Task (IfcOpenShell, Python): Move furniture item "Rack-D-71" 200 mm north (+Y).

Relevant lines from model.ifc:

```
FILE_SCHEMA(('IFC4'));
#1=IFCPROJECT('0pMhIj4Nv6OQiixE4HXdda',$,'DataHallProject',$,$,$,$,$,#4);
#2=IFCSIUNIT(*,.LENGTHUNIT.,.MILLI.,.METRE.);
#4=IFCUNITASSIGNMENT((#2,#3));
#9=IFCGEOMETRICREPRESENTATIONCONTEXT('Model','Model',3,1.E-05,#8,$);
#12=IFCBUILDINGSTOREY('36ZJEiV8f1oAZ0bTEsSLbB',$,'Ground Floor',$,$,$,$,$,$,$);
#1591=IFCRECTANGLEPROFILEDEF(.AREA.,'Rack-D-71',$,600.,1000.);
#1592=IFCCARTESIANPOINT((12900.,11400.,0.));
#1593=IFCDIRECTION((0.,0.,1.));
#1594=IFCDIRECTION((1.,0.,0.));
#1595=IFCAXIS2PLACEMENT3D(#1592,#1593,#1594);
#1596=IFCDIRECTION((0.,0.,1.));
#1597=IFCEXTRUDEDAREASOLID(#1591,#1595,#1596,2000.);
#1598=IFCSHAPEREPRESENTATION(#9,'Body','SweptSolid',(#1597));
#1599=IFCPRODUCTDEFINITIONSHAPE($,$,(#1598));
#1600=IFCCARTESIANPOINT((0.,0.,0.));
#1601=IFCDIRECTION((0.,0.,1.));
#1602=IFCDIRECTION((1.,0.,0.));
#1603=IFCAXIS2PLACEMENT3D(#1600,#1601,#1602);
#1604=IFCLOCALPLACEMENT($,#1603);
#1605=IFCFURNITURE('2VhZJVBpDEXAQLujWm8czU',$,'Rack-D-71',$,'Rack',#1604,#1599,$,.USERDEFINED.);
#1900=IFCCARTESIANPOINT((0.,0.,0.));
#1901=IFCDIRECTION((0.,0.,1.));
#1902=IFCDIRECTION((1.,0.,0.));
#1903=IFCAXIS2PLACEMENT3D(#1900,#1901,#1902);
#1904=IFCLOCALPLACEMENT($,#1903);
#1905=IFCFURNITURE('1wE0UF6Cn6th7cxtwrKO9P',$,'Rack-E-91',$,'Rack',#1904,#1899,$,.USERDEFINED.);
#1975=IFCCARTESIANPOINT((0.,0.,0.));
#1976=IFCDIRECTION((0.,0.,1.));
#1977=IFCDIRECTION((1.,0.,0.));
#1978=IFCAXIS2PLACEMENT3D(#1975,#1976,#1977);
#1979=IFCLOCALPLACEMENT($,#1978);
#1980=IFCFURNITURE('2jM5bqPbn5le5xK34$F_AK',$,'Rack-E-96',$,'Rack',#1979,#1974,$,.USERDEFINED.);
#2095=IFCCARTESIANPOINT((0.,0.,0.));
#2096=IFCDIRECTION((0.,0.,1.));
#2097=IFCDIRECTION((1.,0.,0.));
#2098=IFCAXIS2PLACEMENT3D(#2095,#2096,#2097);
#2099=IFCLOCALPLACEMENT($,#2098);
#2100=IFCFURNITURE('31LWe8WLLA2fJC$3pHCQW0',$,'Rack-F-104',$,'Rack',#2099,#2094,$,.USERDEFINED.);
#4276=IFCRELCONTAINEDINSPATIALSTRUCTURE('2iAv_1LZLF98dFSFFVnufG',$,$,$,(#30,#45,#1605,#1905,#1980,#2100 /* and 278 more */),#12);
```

```python
import ifcopenshell
import ifcopenshell.api.geometry
import ifcopenshell.util.placement
import ifcopenshell.util.unit

model = ifcopenshell.open("model.ifc")
unit_scale = ifcopenshell.util.unit.calculate_unit_scale(model)

item = model.by_guid("2VhZJVBpDEXAQLujWm8czU")
matrix = ifcopenshell.util.placement.get_local_placement(item.ObjectPlacement)
matrix[1, 3] += 0.2 / unit_scale
ifcopenshell.api.geometry.edit_object_placement(model, product=item, matrix=matrix, is_si=False)

print(ifcopenshell.util.placement.get_local_placement(item.ObjectPlacement).round(3) + 0.0)

model.write("model-out.ifc")
```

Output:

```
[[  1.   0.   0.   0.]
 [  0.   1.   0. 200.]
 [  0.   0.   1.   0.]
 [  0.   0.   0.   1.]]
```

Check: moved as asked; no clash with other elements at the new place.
